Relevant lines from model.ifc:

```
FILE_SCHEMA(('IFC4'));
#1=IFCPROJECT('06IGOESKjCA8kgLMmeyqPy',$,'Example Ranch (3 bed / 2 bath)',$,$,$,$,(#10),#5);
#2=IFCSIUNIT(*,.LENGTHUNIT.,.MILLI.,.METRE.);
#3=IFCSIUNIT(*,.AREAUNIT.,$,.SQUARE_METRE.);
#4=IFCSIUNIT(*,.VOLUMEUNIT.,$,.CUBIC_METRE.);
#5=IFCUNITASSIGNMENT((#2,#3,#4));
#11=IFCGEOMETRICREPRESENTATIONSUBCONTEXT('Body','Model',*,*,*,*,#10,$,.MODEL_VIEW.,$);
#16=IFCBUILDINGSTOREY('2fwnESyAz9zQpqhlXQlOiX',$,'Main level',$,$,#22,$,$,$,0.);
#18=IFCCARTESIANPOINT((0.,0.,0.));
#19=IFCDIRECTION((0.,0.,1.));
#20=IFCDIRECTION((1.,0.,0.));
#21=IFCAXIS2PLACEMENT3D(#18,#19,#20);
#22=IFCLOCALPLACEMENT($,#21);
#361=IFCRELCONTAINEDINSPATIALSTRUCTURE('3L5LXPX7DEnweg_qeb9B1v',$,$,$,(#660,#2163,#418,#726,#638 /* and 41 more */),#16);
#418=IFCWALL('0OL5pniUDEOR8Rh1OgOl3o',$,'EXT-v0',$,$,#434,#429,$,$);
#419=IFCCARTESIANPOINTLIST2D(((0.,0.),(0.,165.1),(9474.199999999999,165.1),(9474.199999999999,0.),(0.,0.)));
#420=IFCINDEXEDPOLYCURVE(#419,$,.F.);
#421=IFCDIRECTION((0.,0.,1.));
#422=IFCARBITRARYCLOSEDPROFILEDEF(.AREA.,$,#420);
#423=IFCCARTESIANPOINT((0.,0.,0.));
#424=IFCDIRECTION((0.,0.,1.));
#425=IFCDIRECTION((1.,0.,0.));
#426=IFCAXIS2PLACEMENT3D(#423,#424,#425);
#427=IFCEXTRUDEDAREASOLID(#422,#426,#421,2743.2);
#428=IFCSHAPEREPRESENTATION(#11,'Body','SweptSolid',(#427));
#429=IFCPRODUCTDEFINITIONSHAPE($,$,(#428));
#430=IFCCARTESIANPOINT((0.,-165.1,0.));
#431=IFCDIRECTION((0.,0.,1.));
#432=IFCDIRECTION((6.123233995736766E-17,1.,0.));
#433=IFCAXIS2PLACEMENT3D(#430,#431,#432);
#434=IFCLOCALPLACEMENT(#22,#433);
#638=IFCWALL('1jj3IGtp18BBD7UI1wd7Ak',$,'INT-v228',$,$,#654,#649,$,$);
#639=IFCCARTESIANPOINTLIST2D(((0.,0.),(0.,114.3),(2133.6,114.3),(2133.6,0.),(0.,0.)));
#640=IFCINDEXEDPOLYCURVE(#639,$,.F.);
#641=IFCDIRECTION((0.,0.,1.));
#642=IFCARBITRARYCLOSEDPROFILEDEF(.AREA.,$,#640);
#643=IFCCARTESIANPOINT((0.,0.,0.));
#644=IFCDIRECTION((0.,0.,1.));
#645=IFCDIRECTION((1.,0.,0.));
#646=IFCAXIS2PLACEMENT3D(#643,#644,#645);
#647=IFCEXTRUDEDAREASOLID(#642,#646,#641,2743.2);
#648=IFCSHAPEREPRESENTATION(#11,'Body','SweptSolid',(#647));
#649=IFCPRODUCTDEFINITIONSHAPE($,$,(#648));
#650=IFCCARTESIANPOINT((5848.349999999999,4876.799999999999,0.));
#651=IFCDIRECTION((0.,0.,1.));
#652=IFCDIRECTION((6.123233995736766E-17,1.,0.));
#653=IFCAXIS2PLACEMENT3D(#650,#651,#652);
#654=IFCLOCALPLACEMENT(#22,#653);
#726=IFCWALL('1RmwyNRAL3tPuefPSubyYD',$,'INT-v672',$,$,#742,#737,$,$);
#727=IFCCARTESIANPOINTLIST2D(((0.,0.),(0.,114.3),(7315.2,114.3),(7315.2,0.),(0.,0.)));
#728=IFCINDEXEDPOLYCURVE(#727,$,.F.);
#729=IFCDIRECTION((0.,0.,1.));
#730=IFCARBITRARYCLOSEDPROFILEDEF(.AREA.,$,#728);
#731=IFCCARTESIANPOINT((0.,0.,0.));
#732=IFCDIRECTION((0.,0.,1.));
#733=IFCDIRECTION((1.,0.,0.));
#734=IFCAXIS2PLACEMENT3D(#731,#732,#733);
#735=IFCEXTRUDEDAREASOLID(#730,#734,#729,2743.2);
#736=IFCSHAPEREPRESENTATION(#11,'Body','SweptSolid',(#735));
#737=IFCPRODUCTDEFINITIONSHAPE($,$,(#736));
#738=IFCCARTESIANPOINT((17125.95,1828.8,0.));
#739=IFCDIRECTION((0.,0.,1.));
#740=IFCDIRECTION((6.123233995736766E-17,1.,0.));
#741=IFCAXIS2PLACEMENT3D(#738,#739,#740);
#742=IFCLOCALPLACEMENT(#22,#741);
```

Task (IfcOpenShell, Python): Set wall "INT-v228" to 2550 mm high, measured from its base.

```python
import ifcopenshell
import ifcopenshell.geom
import ifcopenshell.util.representation
import ifcopenshell.util.shape
import ifcopenshell.util.unit

model = ifcopenshell.open("model.ifc")
unit_scale = ifcopenshell.util.unit.calculate_unit_scale(model)
settings = ifcopenshell.geom.settings()


def volume(element):
    """Net volume in cubic metres, openings subtracted."""
    shape = ifcopenshell.geom.create_shape(settings, element)
    return ifcopenshell.util.shape.get_volume(shape.geometry)


wall = model.by_guid("1jj3IGtp18BBD7UI1wd7Ak")
before = volume(wall)

body = ifcopenshell.util.representation.get_representation(wall, "Model", "Body")
solid = body.Items[0]
old_height = solid.Depth
solid.Depth = 2.55 / unit_scale
after = volume(wall)

print(f"height {old_height:g} -> {solid.Depth:g}, volume {before:.3f} -> {after:.3f} m3")

model.write("model_rev.ifc")
```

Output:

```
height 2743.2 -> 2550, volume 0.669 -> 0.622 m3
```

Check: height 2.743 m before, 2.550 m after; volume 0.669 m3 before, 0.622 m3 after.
